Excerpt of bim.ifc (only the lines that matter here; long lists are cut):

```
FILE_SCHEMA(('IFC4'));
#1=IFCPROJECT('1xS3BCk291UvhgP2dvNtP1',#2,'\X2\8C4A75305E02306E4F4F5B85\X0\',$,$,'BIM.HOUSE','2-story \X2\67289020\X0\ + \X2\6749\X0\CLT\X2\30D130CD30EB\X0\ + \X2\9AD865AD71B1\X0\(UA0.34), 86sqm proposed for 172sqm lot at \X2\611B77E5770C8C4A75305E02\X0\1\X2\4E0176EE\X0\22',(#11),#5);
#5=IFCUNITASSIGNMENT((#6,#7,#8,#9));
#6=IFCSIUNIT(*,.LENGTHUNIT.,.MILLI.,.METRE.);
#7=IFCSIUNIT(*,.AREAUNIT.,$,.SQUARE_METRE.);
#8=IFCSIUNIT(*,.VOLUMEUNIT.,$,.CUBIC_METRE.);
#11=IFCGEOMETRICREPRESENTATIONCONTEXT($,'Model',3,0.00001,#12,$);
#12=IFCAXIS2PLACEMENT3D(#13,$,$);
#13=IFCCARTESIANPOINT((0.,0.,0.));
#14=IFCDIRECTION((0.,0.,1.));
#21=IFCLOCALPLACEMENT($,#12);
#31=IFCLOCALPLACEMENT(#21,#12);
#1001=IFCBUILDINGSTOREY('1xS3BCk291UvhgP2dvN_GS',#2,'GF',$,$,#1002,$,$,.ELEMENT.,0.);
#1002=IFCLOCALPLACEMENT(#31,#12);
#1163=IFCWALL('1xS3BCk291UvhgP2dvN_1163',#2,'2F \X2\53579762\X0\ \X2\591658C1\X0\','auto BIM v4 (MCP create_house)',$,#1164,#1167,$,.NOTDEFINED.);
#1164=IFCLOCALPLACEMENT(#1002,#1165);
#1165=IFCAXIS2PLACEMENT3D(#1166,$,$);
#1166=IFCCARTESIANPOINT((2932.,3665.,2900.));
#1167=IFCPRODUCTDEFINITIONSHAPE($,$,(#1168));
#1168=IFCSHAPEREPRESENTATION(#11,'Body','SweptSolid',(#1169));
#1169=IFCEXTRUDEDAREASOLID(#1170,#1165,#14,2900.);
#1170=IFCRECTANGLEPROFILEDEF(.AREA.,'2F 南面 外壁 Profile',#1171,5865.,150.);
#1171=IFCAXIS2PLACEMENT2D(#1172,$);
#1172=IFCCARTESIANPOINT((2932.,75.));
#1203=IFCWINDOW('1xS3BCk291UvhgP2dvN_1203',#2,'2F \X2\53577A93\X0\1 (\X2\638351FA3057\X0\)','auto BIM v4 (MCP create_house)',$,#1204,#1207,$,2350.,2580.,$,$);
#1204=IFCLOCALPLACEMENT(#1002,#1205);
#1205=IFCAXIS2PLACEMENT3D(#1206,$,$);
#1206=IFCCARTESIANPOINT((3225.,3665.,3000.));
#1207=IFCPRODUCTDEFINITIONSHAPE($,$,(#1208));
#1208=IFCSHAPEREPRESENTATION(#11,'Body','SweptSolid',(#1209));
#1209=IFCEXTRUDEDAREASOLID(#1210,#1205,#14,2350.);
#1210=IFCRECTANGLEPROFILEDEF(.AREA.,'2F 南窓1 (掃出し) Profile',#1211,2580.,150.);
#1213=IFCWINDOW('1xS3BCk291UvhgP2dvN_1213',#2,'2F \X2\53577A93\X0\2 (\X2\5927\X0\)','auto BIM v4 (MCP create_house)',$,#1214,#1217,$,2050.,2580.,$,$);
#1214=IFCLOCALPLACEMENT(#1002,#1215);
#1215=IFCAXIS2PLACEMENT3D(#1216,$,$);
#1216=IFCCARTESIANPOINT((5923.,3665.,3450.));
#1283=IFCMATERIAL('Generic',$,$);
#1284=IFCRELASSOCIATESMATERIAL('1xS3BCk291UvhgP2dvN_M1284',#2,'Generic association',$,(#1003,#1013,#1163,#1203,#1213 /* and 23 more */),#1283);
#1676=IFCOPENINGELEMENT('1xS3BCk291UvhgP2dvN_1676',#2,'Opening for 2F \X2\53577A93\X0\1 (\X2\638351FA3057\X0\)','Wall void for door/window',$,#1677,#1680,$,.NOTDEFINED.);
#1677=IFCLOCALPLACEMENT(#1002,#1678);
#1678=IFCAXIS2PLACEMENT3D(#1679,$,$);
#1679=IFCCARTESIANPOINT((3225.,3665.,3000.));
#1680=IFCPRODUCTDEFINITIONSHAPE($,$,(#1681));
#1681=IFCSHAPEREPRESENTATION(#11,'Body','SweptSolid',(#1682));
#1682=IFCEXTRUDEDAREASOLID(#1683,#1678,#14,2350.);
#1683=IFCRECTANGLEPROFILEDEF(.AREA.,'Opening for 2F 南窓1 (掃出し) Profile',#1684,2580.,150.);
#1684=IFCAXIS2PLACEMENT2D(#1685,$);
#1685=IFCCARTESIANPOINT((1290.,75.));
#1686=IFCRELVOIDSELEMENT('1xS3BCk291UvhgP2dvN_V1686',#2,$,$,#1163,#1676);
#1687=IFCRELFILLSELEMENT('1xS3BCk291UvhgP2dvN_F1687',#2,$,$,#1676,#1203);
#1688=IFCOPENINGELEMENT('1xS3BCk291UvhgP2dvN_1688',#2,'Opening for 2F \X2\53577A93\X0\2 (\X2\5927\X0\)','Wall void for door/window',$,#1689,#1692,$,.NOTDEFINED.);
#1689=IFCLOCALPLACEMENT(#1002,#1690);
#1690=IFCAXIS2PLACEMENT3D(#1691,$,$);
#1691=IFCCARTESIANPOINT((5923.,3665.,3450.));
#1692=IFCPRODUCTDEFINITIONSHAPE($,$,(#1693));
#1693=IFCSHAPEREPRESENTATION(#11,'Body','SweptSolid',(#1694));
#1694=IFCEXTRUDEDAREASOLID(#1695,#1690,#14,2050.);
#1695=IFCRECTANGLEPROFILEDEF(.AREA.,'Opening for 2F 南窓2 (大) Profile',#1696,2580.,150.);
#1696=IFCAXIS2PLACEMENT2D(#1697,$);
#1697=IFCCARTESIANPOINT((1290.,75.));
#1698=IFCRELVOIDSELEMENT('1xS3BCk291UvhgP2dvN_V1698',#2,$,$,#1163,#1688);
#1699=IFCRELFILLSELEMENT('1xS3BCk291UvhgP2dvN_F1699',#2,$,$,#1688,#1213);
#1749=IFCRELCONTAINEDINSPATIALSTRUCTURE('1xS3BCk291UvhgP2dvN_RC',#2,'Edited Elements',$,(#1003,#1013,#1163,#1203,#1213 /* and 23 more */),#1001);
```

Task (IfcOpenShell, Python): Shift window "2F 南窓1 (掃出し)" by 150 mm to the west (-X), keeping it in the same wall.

```python
import ifcopenshell
import ifcopenshell.api.geometry
import ifcopenshell.util.placement
import ifcopenshell.util.unit

model = ifcopenshell.open("bim.ifc")
unit_scale = ifcopenshell.util.unit.calculate_unit_scale(model)

window = model.by_id(1203)
opening = window.FillsVoids[0].RelatingOpeningElement
wall = opening.VoidsElements[0].RelatingBuildingElement

wall_matrix = ifcopenshell.util.placement.get_local_placement(wall.ObjectPlacement)
shift = wall_matrix[:3, 0] * -0.15 / unit_scale
before = ifcopenshell.util.placement.get_local_placement(window.ObjectPlacement)[:3, 3].copy()

# The window is not placed relative to its opening, so move both.
for product in (opening, window):
    matrix = ifcopenshell.util.placement.get_local_placement(product.ObjectPlacement)
    matrix[:3, 3] += shift
    ifcopenshell.api.geometry.edit_object_placement(model, product=product, matrix=matrix, is_si=False)

after = ifcopenshell.util.placement.get_local_placement(window.ObjectPlacement)[:3, 3]
print("window moved by", (after - before).round(3) + 0.0)

model.write("bim_updated.ifc")
```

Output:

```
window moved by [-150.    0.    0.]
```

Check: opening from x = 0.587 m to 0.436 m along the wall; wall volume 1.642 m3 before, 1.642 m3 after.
